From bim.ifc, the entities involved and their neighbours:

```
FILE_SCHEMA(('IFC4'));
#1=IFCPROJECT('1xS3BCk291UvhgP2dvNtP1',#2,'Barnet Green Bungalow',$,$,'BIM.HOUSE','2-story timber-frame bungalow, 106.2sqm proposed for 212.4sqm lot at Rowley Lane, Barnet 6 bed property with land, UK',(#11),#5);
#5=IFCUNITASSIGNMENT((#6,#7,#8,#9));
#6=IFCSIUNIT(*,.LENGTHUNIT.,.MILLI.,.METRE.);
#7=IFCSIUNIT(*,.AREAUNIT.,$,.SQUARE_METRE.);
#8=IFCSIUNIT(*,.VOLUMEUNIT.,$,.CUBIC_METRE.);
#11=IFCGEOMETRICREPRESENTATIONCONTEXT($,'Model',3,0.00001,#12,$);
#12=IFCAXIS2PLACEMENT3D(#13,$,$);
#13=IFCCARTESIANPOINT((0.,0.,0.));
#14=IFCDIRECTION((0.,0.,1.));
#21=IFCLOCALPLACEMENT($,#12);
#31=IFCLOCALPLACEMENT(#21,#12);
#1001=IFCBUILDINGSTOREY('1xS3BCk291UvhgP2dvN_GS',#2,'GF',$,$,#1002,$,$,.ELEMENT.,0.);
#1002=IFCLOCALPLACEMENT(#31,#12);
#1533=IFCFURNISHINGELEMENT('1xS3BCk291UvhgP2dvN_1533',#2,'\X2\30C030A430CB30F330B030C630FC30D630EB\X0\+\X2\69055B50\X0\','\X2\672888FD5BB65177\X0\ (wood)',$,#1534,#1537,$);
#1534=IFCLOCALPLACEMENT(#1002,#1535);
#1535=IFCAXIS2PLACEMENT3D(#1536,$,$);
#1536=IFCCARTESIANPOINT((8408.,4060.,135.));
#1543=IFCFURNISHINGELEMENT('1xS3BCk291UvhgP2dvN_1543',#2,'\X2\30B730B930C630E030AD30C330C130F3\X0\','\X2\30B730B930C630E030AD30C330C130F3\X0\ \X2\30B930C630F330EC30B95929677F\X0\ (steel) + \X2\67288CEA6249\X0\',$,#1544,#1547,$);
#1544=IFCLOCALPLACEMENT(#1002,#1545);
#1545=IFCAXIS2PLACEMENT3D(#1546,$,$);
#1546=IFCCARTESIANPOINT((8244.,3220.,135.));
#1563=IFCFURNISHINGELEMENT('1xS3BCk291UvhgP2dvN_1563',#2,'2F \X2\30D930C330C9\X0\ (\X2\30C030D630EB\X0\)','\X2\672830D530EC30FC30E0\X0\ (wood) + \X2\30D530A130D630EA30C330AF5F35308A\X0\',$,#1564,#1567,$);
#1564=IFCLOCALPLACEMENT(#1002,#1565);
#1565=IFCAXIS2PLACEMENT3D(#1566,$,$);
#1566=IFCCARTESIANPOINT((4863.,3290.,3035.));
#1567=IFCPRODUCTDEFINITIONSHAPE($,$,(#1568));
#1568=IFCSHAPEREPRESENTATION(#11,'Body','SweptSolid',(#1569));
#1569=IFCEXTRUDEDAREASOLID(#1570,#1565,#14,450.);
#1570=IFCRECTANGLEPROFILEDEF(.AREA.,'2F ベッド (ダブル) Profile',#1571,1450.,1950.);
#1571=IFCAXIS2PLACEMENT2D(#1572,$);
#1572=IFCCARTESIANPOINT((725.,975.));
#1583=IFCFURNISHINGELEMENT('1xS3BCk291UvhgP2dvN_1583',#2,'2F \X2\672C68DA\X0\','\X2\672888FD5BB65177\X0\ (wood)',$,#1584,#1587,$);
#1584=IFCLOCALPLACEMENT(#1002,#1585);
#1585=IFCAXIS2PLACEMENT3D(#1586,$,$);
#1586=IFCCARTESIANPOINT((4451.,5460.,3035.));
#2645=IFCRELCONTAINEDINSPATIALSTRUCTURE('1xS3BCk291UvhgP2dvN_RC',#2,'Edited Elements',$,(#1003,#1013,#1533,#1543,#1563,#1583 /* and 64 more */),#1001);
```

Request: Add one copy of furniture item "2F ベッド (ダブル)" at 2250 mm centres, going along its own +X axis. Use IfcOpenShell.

```python
import ifcopenshell
import ifcopenshell.api.geometry
import ifcopenshell.api.root
import ifcopenshell.util.element
import ifcopenshell.util.placement
import ifcopenshell.util.unit

model = ifcopenshell.open("bim.ifc")
unit_scale = ifcopenshell.util.unit.calculate_unit_scale(model)


def reuse_history(source, copy):
    """copy_class also copies each property set's owner history, people and application; keep the originals."""
    for rel in copy.IsDefinedBy:
        if rel.is_a("IfcRelDefinesByProperties") and (history := rel.RelatingPropertyDefinition.OwnerHistory):
            rel.RelatingPropertyDefinition.OwnerHistory = source.OwnerHistory
            ifcopenshell.util.element.remove_deep2(model, history)


source = model.by_guid("1xS3BCk291UvhgP2dvN_1563")
base = ifcopenshell.util.placement.get_local_placement(source.ObjectPlacement)
step = base[:3, 0] * 2.25 / unit_scale

for i in range(1, 2):
    copy = ifcopenshell.api.root.copy_class(model, product=source)
    copy.Representation = ifcopenshell.util.element.copy_deep(
        model, source.Representation, exclude=["IfcGeometricRepresentationContext", "IfcRepresentationMap"]
    )
    reuse_history(source, copy)
    matrix = base.copy()
    matrix[:3, 3] += i * step
    print("added at", matrix[:3, 3].round(3) + 0.0)
    ifcopenshell.api.geometry.edit_object_placement(model, product=copy, matrix=matrix, is_si=False)

model.write("bim_updated.ifc")
```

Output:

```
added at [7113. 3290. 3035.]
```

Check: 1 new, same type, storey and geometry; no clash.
